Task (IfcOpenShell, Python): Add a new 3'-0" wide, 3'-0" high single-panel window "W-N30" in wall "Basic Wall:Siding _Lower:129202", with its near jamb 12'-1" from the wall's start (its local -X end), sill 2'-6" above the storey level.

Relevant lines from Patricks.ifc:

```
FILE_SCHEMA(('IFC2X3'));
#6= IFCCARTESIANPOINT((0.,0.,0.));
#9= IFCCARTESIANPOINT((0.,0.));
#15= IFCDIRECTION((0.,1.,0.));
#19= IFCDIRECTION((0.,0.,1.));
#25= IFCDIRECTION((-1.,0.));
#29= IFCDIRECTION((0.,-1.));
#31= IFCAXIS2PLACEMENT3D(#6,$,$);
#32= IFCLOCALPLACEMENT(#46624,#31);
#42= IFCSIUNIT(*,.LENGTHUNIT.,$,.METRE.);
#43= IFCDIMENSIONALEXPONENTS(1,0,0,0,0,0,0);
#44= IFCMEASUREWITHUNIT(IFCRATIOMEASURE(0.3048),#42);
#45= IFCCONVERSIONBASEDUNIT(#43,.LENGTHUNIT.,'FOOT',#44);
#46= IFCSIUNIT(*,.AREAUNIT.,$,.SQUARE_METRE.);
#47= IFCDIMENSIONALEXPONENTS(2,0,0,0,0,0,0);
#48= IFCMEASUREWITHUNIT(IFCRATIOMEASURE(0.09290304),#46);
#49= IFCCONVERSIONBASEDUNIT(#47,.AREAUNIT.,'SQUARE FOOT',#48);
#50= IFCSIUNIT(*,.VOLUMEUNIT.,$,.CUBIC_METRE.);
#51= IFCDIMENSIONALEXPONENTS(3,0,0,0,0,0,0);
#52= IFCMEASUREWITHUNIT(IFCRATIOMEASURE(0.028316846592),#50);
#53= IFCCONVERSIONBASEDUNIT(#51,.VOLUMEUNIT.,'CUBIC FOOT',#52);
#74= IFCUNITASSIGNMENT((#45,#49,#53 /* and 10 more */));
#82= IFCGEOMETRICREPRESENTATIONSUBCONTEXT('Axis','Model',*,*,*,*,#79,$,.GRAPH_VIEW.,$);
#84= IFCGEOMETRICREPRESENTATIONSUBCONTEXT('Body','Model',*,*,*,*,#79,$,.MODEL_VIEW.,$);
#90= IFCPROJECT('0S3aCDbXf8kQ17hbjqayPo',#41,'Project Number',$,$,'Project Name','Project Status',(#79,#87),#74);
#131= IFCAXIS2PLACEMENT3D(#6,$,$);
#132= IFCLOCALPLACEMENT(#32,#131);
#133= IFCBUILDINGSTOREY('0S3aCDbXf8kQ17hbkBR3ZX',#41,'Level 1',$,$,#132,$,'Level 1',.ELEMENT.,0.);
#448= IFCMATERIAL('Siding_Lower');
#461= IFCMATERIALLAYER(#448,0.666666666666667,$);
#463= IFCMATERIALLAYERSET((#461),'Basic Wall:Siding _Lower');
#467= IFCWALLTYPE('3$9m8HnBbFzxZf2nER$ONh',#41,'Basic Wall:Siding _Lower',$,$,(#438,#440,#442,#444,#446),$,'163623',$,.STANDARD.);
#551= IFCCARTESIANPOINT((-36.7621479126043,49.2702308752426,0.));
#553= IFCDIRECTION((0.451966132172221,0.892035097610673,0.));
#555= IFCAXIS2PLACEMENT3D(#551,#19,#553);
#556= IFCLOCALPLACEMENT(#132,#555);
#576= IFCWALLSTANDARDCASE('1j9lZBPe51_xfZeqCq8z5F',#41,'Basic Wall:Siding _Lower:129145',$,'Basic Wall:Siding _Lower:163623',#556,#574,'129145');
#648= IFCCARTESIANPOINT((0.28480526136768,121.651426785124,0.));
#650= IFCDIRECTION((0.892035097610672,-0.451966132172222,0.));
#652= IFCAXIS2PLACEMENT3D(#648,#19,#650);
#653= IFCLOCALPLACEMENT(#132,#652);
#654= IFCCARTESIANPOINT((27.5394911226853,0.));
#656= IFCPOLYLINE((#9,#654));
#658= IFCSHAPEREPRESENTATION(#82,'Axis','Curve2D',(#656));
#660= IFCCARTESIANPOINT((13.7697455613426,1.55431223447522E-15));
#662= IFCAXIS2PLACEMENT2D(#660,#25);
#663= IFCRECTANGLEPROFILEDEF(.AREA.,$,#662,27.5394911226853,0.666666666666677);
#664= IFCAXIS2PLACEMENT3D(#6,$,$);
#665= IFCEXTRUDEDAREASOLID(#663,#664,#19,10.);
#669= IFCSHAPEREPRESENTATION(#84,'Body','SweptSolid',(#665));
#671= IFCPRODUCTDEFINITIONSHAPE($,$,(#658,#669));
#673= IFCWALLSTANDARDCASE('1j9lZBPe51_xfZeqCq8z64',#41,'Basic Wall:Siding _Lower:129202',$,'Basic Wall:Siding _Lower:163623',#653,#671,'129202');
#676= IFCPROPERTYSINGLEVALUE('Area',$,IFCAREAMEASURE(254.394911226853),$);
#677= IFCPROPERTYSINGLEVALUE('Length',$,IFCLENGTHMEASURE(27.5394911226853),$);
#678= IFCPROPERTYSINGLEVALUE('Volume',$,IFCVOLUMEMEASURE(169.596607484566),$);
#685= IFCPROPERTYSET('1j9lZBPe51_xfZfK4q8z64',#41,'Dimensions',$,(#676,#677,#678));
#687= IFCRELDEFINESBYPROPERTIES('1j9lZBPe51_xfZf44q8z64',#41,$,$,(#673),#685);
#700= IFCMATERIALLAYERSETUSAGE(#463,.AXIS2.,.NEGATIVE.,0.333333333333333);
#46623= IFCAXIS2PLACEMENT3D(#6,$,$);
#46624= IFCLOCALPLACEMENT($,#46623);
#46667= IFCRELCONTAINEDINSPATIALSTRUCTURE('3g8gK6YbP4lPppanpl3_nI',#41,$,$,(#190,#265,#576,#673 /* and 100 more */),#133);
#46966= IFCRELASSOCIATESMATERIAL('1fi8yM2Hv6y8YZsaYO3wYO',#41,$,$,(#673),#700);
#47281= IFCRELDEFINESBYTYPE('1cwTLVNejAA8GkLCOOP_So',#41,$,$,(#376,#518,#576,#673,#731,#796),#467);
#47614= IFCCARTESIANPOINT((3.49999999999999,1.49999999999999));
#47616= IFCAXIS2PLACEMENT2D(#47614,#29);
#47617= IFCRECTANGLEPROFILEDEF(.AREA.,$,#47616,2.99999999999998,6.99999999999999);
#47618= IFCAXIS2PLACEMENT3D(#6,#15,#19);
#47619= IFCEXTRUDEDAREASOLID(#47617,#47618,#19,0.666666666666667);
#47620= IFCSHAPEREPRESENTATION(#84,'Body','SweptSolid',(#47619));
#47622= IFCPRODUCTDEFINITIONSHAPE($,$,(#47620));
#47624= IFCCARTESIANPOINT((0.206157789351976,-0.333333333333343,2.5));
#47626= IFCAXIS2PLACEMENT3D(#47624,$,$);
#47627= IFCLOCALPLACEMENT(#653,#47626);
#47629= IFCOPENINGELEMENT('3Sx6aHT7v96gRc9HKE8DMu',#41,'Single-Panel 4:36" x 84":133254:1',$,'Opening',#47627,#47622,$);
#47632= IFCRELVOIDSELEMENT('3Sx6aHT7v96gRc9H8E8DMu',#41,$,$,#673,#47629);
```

```python
import numpy as np
import ifcopenshell
import ifcopenshell.api.feature
import ifcopenshell.api.geometry
import ifcopenshell.api.pset
import ifcopenshell.api.root
import ifcopenshell.api.spatial
import ifcopenshell.api.type
import ifcopenshell.geom
import ifcopenshell.util.element
import ifcopenshell.util.placement
import ifcopenshell.util.representation
import ifcopenshell.util.shape
import ifcopenshell.util.unit

model = ifcopenshell.open("Patricks.ifc")
unit_scale = ifcopenshell.util.unit.calculate_unit_scale(model)
area_scale = ifcopenshell.util.unit.calculate_unit_scale(model, "AREAUNIT")
volume_scale = ifcopenshell.util.unit.calculate_unit_scale(model, "VOLUMEUNIT")
settings = ifcopenshell.geom.settings()


def volume(element):
    """Net volume in cubic metres, openings subtracted."""
    shape = ifcopenshell.geom.create_shape(settings, element)
    return ifcopenshell.util.shape.get_volume(shape.geometry)


wall = model.by_guid("1j9lZBPe51_xfZeqCq8z64")
storey = ifcopenshell.util.element.get_container(wall, ifc_class="IfcBuildingStorey")
context = ifcopenshell.util.representation.get_context(model, "Model", "Body", "MODEL_VIEW")
before = volume(wall)

width, height, from_end, sill = 0.9144, 0.9144, 3.683, 0.762  # metres

# The wall runs along its own X axis, and the end named is its -X end.
wall_shape = ifcopenshell.geom.create_shape(settings, wall)
x, y, z = ifcopenshell.util.shape.get_vertices(wall_shape.geometry).T
start = x.min() + from_end
face, thickness = float(y.min()), float(y.max() - y.min())
wall_matrix = ifcopenshell.util.placement.get_local_placement(wall.ObjectPlacement)
level = ifcopenshell.util.placement.get_local_placement(storey.ObjectPlacement)[2, 3]


def in_wall(x, y):
    """Placement at x, y metres in the wall's axes, at sill height."""
    matrix = wall_matrix.copy()
    matrix[:, 3] = wall_matrix @ np.array([x / unit_scale, y / unit_scale, 0.0, 1.0])
    matrix[2, 3] = level + sill / unit_scale
    return matrix


# Opening: a box that overshoots both wall faces by 50 mm.
opening = ifcopenshell.api.root.create_entity(model, ifc_class="IfcOpeningElement")
box = ifcopenshell.api.geometry.add_wall_representation(
    model, context=context, length=width, height=height, thickness=thickness + 0.1
)
ifcopenshell.api.geometry.assign_representation(model, product=opening, representation=box)
ifcopenshell.api.geometry.edit_object_placement(model, product=opening, matrix=in_wall(start, face - 0.05), is_si=False)
ifcopenshell.api.feature.add_feature(model, feature=opening, element=wall)

window = ifcopenshell.api.root.create_entity(model, ifc_class="IfcWindow", name="W-N30")
window.OverallWidth, window.OverallHeight = width / unit_scale, height / unit_scale
body = ifcopenshell.api.geometry.add_window_representation(
    model,
    context=context,
    overall_width=window.OverallWidth,
    overall_height=window.OverallHeight,
    partition_type="SINGLE_PANEL",
)
ifcopenshell.api.geometry.assign_representation(model, product=window, representation=body)
ifcopenshell.api.spatial.assign_container(model, products=[window], relating_structure=storey)
fills = ifcopenshell.api.feature.add_filling(model, opening=opening, element=window)
fills.OwnerHistory = window.OwnerHistory  # required in IFC2X3

# IFC2X3 keeps the operation on the window style.
style = ifcopenshell.api.root.create_entity(model, ifc_class="IfcWindowStyle", name="W-N30")
style.OperationType, style.ConstructionType = "SINGLE_PANEL", "NOTDEFINED"
style.ParameterTakesPrecedence = style.Sizeable = False
ifcopenshell.api.type.assign_type(model, related_objects=[window], relating_type=style)

# Centre the window in the wall's thickness.
ifcopenshell.api.geometry.edit_object_placement(model, product=window, matrix=in_wall(start, face), is_si=False)
window_shape = ifcopenshell.geom.create_shape(settings, window)
depth = ifcopenshell.util.shape.get_vertices(window_shape.geometry)[:, 1]
offset = face + thickness / 2 - (depth.min() + depth.max()) / 2
ifcopenshell.api.geometry.edit_object_placement(model, product=window, matrix=in_wall(start, offset), is_si=False)

after = volume(wall)

# Update the wall's stored quantities.
pset = model.by_id(ifcopenshell.util.element.get_pset(wall, "Dimensions", should_inherit=False)["id"])
ifcopenshell.api.pset.edit_pset(model, pset=pset, properties={
    "Area": model.create_entity("IfcAreaMeasure", after / thickness / area_scale),
    "Volume": model.create_entity("IfcVolumeMeasure", after / volume_scale),
})

print(f"wall volume {before:.3f} -> {after:.3f} m3")

model.write("Patricks_edited.ifc")
```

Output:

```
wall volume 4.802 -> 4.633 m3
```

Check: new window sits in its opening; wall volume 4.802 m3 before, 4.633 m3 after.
